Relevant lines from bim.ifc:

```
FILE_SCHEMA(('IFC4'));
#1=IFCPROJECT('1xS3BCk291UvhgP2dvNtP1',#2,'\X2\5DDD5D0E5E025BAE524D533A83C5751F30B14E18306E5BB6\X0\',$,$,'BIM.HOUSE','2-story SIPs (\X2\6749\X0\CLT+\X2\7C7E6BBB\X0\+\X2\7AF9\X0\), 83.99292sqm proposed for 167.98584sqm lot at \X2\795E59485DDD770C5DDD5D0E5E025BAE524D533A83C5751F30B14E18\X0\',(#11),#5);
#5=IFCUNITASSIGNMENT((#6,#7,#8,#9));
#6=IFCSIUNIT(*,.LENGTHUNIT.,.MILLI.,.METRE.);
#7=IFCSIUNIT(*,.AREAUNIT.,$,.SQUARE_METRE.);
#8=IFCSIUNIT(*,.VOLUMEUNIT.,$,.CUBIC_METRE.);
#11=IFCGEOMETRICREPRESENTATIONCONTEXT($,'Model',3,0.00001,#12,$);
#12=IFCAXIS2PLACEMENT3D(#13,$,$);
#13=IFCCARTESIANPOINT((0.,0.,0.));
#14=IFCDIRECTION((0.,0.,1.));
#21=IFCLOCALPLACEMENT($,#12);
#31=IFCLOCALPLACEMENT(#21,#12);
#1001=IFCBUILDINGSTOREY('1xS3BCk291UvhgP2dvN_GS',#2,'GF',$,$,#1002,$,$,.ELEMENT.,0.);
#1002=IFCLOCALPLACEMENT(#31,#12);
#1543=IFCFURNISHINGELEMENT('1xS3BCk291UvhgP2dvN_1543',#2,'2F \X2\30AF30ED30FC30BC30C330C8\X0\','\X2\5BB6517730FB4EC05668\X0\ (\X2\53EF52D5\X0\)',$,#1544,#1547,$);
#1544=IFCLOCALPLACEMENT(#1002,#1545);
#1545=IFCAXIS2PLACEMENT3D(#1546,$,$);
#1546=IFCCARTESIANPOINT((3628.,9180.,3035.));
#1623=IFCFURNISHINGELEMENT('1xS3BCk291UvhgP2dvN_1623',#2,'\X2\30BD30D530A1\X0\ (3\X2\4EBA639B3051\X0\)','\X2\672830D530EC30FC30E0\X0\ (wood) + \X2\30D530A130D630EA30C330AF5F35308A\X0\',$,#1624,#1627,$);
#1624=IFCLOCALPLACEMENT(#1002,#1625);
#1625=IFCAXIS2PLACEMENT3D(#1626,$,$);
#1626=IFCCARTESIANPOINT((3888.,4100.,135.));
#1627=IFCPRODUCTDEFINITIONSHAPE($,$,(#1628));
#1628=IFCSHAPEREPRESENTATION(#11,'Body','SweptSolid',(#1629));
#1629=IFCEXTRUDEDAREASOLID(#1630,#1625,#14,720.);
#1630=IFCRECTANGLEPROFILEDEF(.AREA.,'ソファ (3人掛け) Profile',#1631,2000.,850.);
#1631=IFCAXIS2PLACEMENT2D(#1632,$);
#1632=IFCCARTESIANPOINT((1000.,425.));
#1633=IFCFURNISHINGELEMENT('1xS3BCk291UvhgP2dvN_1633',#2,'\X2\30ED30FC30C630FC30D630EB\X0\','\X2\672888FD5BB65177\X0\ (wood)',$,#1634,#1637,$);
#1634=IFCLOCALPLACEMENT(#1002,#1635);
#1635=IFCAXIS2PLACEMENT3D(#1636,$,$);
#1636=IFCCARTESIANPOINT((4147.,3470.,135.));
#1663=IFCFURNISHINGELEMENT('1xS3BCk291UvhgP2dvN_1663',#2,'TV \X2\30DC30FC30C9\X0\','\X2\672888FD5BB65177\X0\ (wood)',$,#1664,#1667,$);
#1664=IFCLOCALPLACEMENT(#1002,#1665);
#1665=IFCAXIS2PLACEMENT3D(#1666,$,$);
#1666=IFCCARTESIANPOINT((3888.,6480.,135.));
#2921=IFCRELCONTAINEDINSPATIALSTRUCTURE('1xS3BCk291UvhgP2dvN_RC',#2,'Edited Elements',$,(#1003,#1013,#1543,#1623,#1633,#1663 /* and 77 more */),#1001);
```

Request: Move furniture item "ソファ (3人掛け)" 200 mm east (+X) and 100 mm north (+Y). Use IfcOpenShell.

```python
import ifcopenshell
import ifcopenshell.api.geometry
import ifcopenshell.util.placement
import ifcopenshell.util.unit

model = ifcopenshell.open("bim.ifc")
unit_scale = ifcopenshell.util.unit.calculate_unit_scale(model)

item = model.by_id(1623)
matrix = ifcopenshell.util.placement.get_local_placement(item.ObjectPlacement)
matrix[0, 3] += 0.2 / unit_scale
matrix[1, 3] += 0.1 / unit_scale
ifcopenshell.api.geometry.edit_object_placement(model, product=item, matrix=matrix, is_si=False)

print(ifcopenshell.util.placement.get_local_placement(item.ObjectPlacement).round(3) + 0.0)

model.write("bim_v2.ifc")
```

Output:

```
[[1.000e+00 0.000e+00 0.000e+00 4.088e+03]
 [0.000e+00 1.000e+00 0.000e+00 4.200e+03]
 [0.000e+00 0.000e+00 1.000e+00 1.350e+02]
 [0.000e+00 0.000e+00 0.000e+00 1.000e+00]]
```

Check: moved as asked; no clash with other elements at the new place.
